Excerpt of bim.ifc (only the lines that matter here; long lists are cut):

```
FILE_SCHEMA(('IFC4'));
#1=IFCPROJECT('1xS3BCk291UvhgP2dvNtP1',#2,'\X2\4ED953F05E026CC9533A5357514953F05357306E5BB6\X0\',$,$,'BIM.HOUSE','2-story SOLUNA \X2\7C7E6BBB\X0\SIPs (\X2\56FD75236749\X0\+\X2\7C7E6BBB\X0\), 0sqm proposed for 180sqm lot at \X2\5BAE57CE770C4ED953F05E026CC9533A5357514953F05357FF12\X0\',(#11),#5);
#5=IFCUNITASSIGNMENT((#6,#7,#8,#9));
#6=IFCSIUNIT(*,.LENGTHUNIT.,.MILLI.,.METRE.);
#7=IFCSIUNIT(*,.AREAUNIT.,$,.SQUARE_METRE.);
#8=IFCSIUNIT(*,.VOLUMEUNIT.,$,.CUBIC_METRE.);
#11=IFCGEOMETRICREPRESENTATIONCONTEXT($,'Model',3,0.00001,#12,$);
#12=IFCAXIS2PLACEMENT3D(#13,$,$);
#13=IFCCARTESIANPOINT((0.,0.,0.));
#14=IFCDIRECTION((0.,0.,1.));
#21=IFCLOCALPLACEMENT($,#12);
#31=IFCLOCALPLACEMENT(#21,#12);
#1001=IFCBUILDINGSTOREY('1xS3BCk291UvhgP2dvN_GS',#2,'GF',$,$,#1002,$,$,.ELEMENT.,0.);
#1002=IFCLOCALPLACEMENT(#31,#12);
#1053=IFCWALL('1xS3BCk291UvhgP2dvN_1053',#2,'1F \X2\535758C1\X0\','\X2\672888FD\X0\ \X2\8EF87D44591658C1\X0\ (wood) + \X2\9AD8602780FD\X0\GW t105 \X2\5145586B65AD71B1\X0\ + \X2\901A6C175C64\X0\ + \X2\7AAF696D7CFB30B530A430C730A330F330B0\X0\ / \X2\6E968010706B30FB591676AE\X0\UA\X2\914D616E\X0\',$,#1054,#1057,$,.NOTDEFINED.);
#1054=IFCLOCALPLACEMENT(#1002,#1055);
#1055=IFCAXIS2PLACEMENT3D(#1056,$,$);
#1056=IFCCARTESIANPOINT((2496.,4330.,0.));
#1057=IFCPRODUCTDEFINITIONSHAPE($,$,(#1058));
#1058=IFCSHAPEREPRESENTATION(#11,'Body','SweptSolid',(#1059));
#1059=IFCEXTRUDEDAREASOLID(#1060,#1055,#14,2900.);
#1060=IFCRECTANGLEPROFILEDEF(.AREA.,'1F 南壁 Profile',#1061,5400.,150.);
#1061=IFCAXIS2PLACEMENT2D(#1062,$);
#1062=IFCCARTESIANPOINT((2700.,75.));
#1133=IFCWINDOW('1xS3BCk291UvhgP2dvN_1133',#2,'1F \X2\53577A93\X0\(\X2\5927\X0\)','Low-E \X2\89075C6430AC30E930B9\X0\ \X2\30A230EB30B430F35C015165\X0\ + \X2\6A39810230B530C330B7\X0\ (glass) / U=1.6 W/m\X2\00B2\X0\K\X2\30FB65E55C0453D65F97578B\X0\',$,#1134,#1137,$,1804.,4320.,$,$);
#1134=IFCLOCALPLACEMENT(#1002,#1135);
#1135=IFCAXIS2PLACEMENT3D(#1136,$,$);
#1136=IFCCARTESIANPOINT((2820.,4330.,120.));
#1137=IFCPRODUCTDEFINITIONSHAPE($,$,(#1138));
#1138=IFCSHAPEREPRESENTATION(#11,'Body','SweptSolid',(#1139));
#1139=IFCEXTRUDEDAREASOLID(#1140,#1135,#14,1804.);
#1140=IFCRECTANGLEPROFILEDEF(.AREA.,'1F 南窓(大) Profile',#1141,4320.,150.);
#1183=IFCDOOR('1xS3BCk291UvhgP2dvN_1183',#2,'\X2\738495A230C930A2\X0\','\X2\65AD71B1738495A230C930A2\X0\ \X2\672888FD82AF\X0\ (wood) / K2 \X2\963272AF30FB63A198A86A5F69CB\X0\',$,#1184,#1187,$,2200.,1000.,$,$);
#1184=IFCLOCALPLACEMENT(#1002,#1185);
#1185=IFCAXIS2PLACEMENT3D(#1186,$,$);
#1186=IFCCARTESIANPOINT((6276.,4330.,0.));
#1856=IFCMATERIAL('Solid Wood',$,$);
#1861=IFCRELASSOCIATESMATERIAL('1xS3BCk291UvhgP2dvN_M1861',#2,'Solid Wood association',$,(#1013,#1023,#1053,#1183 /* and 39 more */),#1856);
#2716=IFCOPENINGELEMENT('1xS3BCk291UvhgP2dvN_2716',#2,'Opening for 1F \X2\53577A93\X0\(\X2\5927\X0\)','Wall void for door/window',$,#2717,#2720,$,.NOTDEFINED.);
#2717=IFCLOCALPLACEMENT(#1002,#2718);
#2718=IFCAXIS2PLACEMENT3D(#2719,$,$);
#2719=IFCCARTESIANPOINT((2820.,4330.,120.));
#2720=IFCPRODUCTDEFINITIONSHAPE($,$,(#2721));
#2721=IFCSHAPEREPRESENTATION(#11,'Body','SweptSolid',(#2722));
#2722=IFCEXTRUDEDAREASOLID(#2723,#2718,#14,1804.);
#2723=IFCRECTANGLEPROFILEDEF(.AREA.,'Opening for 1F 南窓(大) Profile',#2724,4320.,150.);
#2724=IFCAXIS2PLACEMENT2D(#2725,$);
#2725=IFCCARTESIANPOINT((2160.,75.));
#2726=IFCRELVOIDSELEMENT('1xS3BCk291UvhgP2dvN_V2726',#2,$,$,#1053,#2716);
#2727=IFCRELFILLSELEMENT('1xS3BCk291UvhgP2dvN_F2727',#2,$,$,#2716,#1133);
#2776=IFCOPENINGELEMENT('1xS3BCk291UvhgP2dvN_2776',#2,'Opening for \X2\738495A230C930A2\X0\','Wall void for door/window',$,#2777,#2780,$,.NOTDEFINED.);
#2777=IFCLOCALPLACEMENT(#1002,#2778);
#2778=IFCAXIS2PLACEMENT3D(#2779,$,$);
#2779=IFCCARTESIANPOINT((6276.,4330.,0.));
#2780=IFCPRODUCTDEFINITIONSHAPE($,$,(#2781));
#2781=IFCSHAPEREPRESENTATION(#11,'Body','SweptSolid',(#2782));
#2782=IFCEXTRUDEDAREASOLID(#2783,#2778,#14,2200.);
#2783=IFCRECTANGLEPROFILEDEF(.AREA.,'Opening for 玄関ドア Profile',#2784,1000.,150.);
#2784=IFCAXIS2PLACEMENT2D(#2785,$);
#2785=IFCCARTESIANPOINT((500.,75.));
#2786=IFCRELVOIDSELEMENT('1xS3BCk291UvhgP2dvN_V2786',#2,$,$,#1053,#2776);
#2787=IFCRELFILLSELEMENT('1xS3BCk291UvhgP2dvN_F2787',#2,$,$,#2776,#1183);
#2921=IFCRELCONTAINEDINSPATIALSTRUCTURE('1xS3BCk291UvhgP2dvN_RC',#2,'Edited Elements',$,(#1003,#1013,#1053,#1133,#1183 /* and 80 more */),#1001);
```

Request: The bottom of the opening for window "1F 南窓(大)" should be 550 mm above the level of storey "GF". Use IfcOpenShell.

```python
import numpy as np
import ifcopenshell
import ifcopenshell.api.geometry
import ifcopenshell.geom
import ifcopenshell.util.element
import ifcopenshell.util.placement
import ifcopenshell.util.shape
import ifcopenshell.util.unit

model = ifcopenshell.open("bim.ifc")
unit_scale = ifcopenshell.util.unit.calculate_unit_scale(model)

window = model.by_guid("1xS3BCk291UvhgP2dvN_1133")
opening = window.FillsVoids[0].RelatingOpeningElement
storey = ifcopenshell.util.element.get_container(window, ifc_class="IfcBuildingStorey")
level = ifcopenshell.util.placement.get_local_placement(storey.ObjectPlacement)[2, 3]

# The opening's origin need not be at the sill, so measure its lowest point.
shape = ifcopenshell.geom.create_shape(ifcopenshell.geom.settings(), opening)
bottom = ifcopenshell.util.shape.get_shape_bottom_elevation(shape, shape.geometry) / unit_scale
dz = level + 550.0 - bottom

shift = np.array([0.0, 0.0, dz])
# The window is not placed relative to its opening, so move both.
for product in (opening, window):
    matrix = ifcopenshell.util.placement.get_local_placement(product.ObjectPlacement)
    matrix[:3, 3] += shift
    ifcopenshell.api.geometry.edit_object_placement(model, product=product, matrix=matrix, is_si=False)

print(f"moved by {dz * unit_scale:+.3f} m")

model.write("bim_edited.ifc")
```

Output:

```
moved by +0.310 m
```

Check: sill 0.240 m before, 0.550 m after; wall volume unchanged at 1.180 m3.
